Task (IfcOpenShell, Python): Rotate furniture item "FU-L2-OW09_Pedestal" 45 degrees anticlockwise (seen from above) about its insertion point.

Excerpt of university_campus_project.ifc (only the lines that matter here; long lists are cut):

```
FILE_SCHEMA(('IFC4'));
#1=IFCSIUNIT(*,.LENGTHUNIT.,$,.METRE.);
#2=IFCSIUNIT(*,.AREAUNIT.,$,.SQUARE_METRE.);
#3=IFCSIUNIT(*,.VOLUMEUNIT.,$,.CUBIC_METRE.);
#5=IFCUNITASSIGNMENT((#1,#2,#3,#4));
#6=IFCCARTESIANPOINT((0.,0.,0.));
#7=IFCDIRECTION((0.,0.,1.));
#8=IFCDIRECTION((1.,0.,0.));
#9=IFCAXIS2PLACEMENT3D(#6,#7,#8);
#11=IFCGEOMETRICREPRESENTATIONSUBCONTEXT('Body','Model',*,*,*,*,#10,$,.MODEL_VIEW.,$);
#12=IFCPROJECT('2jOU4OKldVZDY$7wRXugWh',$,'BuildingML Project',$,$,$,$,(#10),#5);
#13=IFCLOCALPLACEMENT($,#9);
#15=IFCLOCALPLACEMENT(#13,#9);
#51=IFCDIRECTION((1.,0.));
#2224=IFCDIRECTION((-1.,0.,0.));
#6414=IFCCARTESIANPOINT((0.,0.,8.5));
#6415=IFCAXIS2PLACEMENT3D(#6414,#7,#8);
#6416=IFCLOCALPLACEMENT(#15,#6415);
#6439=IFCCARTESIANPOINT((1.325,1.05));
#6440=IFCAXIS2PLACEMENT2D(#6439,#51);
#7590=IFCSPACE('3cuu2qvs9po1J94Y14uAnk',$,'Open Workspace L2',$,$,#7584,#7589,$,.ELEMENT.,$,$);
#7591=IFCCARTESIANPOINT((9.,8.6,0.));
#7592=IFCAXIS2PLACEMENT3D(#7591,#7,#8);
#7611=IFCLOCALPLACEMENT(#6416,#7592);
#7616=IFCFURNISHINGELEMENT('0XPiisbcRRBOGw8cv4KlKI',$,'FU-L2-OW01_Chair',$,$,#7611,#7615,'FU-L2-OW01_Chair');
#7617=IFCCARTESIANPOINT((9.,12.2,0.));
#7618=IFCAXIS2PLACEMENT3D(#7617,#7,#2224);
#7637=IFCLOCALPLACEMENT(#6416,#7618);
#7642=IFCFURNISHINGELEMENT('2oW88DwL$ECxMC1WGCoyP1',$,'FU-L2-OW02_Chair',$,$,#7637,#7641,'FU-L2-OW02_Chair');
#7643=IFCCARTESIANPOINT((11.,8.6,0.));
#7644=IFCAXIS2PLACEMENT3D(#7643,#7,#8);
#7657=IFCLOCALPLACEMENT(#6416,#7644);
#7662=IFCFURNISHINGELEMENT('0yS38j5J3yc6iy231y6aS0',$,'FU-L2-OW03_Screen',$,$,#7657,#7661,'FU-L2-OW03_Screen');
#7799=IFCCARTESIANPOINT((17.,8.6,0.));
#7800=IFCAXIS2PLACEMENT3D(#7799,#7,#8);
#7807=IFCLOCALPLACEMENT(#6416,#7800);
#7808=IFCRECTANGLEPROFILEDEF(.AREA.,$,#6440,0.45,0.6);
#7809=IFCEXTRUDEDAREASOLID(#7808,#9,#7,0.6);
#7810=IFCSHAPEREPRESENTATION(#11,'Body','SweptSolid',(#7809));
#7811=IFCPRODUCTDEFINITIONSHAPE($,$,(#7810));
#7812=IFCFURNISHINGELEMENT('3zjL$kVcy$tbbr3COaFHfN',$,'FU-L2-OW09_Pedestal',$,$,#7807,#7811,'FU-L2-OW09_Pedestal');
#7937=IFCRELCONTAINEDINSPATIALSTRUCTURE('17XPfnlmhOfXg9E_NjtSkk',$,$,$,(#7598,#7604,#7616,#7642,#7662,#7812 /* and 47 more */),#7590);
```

```python
import ifcopenshell
import ifcopenshell.api.geometry
import ifcopenshell.util.placement

model = ifcopenshell.open("university_campus_project.ifc")

item = model.by_guid("3zjL$kVcy$tbbr3COaFHfN")
matrix = ifcopenshell.util.placement.get_local_placement(item.ObjectPlacement)
matrix = matrix @ ifcopenshell.util.placement.rotation(45, "Z")
ifcopenshell.api.geometry.edit_object_placement(model, product=item, matrix=matrix, is_si=False)

print(ifcopenshell.util.placement.get_local_placement(item.ObjectPlacement).round(3) + 0.0)

model.write("university_campus_project_v2.ifc")
```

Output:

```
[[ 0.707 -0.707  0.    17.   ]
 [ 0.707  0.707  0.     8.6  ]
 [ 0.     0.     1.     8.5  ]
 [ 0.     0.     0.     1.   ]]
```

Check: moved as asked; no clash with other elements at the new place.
